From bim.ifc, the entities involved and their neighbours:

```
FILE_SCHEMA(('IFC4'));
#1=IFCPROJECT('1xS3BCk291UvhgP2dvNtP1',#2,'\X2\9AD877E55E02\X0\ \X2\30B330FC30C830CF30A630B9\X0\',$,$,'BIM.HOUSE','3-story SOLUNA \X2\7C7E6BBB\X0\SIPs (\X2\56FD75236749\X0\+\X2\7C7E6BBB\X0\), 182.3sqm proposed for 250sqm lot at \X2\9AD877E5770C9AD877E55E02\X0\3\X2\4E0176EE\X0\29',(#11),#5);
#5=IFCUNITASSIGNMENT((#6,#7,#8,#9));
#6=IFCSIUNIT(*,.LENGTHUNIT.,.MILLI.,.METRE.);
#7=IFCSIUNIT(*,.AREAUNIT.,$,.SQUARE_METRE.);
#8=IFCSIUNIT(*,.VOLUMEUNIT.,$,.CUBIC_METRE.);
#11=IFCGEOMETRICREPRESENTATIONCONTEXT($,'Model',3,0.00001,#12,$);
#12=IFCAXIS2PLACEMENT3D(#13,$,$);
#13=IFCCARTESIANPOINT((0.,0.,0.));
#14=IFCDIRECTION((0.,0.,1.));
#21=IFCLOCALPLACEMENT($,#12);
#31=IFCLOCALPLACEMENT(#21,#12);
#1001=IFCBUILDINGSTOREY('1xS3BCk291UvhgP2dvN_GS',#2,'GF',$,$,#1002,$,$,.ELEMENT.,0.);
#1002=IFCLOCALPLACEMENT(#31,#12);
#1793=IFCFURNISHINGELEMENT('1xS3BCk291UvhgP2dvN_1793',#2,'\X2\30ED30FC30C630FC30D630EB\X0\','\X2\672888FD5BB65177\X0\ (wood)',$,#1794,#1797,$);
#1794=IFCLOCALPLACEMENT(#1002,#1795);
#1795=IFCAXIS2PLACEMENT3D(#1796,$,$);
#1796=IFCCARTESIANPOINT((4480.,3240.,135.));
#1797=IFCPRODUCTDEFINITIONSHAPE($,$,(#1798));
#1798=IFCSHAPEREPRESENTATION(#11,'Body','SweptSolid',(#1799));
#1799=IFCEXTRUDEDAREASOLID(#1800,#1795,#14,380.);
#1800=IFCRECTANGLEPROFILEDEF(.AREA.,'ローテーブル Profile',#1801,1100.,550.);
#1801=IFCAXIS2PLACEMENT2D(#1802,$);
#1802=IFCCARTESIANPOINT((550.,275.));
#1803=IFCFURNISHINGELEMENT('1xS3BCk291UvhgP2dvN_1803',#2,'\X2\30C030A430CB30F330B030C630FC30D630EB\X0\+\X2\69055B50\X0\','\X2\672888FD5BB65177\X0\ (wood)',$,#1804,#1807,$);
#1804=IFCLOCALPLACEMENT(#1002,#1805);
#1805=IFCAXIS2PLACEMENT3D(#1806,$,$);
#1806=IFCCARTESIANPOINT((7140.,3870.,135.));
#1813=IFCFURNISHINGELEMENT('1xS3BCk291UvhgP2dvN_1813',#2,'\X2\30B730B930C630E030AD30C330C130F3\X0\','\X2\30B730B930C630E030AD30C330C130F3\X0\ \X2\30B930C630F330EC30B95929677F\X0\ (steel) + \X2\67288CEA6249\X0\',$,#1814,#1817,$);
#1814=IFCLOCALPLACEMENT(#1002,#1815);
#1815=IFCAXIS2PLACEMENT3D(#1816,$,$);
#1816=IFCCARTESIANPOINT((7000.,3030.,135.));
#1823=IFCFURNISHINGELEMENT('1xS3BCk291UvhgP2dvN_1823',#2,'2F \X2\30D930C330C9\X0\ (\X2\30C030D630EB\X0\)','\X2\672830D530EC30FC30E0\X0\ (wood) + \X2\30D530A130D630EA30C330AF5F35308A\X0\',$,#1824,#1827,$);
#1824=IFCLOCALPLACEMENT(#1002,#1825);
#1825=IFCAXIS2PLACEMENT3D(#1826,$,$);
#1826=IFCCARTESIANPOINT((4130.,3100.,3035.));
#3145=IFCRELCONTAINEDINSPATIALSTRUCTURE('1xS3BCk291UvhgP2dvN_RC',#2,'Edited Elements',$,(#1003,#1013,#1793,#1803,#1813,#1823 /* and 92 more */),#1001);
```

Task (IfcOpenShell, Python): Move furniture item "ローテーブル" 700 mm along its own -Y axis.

```python
import ifcopenshell
import ifcopenshell.api.geometry
import ifcopenshell.util.placement
import ifcopenshell.util.unit

model = ifcopenshell.open("bim.ifc")
unit_scale = ifcopenshell.util.unit.calculate_unit_scale(model)

item = model.by_id(1793)
matrix = ifcopenshell.util.placement.get_local_placement(item.ObjectPlacement)
matrix[:3, 3] -= matrix[:3, 1] * 0.7 / unit_scale
ifcopenshell.api.geometry.edit_object_placement(model, product=item, matrix=matrix, is_si=False)

print(ifcopenshell.util.placement.get_local_placement(item.ObjectPlacement).round(3) + 0.0)

model.write("bim-out.ifc")
```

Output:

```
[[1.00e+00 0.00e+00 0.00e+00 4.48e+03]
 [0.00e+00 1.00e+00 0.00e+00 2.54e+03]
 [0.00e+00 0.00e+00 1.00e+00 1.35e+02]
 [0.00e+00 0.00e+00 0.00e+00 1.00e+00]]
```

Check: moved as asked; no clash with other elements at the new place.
